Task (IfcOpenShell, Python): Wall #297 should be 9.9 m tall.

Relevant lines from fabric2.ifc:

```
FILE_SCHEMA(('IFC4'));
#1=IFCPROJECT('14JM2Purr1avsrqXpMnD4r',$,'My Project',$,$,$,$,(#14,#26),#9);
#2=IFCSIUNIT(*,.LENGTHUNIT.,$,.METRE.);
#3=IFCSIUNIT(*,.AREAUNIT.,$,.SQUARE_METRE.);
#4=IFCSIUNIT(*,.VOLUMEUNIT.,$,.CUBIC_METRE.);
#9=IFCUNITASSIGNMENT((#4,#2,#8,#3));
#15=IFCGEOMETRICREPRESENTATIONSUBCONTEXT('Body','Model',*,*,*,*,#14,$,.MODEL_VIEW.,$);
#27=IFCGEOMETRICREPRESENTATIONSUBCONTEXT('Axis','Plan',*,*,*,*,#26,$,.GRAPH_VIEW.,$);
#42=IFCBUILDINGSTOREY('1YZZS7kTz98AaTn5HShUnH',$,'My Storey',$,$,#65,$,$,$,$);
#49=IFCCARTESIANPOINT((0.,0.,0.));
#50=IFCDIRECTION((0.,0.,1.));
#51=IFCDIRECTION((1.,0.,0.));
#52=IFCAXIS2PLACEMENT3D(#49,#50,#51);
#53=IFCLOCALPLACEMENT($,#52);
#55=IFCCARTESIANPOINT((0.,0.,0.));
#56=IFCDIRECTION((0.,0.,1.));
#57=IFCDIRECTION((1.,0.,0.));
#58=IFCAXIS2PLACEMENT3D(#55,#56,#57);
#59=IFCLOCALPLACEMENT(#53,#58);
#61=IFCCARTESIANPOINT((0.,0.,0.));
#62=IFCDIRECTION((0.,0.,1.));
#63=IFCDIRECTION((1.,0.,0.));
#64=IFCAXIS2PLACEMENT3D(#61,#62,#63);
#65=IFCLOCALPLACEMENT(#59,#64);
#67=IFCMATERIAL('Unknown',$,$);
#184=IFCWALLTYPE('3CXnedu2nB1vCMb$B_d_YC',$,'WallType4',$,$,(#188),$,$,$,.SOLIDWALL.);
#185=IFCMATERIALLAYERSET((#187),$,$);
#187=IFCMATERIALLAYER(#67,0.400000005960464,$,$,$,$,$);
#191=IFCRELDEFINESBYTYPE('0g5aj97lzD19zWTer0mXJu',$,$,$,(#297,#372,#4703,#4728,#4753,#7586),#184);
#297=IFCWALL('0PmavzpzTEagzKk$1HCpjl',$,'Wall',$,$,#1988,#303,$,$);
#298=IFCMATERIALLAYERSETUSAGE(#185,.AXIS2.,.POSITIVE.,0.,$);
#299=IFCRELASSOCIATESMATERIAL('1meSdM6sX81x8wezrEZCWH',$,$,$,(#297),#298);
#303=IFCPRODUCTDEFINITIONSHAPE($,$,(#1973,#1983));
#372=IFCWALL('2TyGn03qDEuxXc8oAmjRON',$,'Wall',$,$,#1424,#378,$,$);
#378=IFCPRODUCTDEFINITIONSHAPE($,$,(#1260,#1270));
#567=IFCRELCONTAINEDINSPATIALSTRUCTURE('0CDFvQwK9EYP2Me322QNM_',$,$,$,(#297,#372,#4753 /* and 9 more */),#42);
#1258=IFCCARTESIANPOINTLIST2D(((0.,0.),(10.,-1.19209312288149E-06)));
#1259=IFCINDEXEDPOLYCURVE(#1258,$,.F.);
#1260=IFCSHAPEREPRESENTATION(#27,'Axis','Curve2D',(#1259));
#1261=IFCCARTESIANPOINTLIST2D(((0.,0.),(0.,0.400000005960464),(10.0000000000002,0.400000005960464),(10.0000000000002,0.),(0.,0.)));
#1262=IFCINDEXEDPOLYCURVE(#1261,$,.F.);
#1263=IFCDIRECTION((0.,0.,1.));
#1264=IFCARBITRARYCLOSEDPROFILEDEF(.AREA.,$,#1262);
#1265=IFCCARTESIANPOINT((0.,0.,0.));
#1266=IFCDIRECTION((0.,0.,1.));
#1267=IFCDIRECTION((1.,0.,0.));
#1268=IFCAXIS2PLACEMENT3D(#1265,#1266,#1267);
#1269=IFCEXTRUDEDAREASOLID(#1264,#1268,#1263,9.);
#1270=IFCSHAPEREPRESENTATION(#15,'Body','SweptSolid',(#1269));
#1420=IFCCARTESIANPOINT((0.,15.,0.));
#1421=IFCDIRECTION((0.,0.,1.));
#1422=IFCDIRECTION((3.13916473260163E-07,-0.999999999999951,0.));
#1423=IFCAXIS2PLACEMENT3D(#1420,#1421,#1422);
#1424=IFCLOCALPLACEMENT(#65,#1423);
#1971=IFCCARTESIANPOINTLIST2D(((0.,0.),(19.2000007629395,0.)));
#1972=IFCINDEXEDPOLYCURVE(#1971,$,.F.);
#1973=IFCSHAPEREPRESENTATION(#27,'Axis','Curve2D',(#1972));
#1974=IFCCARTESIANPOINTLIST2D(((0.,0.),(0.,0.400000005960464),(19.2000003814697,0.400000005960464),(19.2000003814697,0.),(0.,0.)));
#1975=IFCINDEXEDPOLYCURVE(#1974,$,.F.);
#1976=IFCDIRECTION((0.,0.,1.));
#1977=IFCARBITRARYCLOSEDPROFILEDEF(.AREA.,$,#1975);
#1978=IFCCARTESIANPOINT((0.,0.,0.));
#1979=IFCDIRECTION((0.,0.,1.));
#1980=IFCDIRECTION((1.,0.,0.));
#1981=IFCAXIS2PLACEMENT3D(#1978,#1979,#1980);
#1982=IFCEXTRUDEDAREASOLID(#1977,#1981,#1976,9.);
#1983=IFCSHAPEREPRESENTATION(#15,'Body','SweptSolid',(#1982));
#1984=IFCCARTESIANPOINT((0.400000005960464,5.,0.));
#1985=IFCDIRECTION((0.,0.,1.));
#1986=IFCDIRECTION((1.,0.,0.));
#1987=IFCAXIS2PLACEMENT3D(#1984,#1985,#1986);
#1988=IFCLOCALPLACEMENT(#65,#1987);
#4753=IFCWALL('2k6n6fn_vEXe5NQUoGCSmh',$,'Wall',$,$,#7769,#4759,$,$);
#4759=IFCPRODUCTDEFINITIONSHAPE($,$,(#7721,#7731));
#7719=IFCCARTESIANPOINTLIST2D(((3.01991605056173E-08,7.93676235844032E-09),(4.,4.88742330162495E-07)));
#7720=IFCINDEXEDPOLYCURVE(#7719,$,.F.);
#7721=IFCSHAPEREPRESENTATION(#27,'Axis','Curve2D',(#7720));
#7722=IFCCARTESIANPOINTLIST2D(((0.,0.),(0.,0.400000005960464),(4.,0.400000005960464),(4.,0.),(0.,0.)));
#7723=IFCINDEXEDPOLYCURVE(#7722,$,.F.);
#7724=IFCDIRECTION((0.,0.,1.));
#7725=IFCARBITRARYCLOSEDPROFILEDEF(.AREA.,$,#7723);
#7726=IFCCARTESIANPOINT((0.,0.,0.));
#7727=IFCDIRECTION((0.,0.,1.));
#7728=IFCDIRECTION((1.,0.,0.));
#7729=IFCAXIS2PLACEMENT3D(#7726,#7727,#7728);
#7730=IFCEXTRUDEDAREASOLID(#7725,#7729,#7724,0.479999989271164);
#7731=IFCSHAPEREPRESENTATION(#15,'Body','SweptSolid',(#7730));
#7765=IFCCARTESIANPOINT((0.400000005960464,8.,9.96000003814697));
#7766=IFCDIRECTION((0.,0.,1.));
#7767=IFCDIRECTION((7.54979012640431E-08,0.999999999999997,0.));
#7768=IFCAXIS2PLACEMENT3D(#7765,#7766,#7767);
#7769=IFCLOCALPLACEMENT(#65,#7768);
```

```python
import ifcopenshell
import ifcopenshell.geom
import ifcopenshell.util.representation
import ifcopenshell.util.shape

model = ifcopenshell.open("fabric2.ifc")
settings = ifcopenshell.geom.settings()


def volume(element):
    """Net volume in cubic metres, openings subtracted."""
    shape = ifcopenshell.geom.create_shape(settings, element)
    return ifcopenshell.util.shape.get_volume(shape.geometry)


wall = model.by_guid("0PmavzpzTEagzKk$1HCpjl")
before = volume(wall)

body = ifcopenshell.util.representation.get_representation(wall, "Model", "Body")
solid = body.Items[0]
old_height = solid.Depth
solid.Depth = 9.9
after = volume(wall)

print(f"height {old_height:g} -> {solid.Depth:g}, volume {before:.3f} -> {after:.3f} m3")

model.write("fabric2_rev.ifc")
```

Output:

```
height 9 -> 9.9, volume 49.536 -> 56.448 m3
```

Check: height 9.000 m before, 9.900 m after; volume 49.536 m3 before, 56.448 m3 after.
